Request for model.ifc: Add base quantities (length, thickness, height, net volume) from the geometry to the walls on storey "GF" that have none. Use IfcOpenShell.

First a look at what the model holds.

```python
import ifcopenshell
import ifcopenshell.util.element
import ifcopenshell.util.unit

model = ifcopenshell.open("model.ifc")
print(model.schema)
for unit_type in ("LENGTHUNIT", "AREAUNIT", "VOLUMEUNIT"):
    print(unit_type, ifcopenshell.util.unit.calculate_unit_scale(model, unit_type))
storey = next(s for s in model.by_type("IfcBuildingStorey") if s.Name == "GF")
walls = [e for e in ifcopenshell.util.element.get_decomposition(storey) if e.is_a("IfcWall")]
for e in sorted(walls, key=lambda e: e.id()):
    print(e.id(), e.is_a(), e.Name, list(ifcopenshell.util.element.get_psets(e, qtos_only=True)), sep=" | ")
```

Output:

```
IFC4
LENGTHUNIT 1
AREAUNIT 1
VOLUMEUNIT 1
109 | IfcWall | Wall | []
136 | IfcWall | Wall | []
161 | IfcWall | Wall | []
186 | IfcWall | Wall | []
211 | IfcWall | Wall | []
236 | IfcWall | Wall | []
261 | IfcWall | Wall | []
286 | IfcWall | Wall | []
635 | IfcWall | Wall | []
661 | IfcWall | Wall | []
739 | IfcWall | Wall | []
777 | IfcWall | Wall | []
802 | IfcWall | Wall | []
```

```python
import ifcopenshell
import ifcopenshell.api.pset
import ifcopenshell.geom
import ifcopenshell.util.element
import ifcopenshell.util.shape
import ifcopenshell.util.unit

model = ifcopenshell.open("model.ifc")
unit_scale = ifcopenshell.util.unit.calculate_unit_scale(model)
volume_scale = ifcopenshell.util.unit.calculate_unit_scale(model, "VOLUMEUNIT")
settings = ifcopenshell.geom.settings()

storey = next(s for s in model.by_type("IfcBuildingStorey") if s.Name == "GF")
walls = [e for e in ifcopenshell.util.element.get_decomposition(storey) if e.is_a("IfcWall")]

for e in sorted(walls, key=lambda e: e.id()):
    if ifcopenshell.util.element.get_psets(e, qtos_only=True, should_inherit=False):
        continue
    # Geometry comes back in metres, in the element's own axes.
    shape = ifcopenshell.geom.create_shape(settings, e)
    values = {
        "Length": ifcopenshell.util.shape.get_x(shape.geometry) / unit_scale,
        "Width": ifcopenshell.util.shape.get_y(shape.geometry) / unit_scale,
        "Height": ifcopenshell.util.shape.get_z(shape.geometry) / unit_scale,
        "NetVolume": ifcopenshell.util.shape.get_volume(shape.geometry) / volume_scale,
    }
    qto = ifcopenshell.api.pset.add_qto(model, product=e, name="Qto_WallBaseQuantities")
    ifcopenshell.api.pset.edit_qto(model, qto=qto, properties=values)
    print(e.id(), {k: round(v, 3) for k, v in values.items()})

model.write("model_rev.ifc")
```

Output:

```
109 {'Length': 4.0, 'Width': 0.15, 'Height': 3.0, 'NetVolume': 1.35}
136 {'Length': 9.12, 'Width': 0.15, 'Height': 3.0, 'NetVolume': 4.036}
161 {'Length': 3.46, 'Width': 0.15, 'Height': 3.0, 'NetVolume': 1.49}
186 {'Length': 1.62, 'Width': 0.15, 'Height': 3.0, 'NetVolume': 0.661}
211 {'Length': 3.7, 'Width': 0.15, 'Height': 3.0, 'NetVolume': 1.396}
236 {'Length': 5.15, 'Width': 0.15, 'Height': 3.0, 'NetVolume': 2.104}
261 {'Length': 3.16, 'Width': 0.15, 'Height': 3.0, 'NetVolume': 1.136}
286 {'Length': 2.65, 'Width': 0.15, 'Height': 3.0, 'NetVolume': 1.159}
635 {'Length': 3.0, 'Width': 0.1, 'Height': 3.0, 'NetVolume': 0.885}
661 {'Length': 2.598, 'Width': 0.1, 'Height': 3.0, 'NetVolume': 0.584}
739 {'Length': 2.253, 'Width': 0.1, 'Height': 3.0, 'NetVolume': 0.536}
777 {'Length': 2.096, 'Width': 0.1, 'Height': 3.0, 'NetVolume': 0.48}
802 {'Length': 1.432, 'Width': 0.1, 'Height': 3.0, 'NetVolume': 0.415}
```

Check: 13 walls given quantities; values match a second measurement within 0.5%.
